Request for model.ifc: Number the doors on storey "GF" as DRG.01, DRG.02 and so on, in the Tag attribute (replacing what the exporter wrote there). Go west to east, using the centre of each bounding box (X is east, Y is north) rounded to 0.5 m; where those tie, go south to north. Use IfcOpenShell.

First a look at what the model holds.

```python
import ifcopenshell
import ifcopenshell.util.element
import ifcopenshell.util.placement

model = ifcopenshell.open("model.ifc")
print(model.schema)
storey = next(s for s in model.by_type("IfcBuildingStorey") if s.Name == "GF")
doors = [e for e in ifcopenshell.util.element.get_decomposition(storey) if e.is_a("IfcDoor")]
for e in sorted(doors, key=lambda e: e.id()):
    origin = ifcopenshell.util.placement.get_local_placement(e.ObjectPlacement)[:3, 3]
    print(e.id(), e.Tag, e.Name, origin.round(2) + 0.0, sep=" | ")
```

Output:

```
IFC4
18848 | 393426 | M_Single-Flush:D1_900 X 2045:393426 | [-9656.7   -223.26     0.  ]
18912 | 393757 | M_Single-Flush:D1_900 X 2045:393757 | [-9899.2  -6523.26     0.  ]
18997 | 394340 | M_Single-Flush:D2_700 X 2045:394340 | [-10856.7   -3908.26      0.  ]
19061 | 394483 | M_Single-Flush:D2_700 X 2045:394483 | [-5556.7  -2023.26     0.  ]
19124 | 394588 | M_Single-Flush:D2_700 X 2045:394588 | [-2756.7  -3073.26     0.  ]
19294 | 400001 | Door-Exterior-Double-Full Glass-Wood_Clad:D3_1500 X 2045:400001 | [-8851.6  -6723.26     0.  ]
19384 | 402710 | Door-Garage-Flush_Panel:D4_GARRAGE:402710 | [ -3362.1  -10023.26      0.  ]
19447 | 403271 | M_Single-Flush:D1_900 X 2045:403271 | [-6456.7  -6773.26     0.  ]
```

```python
import ifcopenshell
import ifcopenshell.geom
import ifcopenshell.util.element
import ifcopenshell.util.shape

model = ifcopenshell.open("model.ifc")
settings = ifcopenshell.geom.settings()
settings.set("use-world-coords", True)


def centre(element):
    shape = ifcopenshell.geom.create_shape(settings, element)
    return ifcopenshell.util.shape.get_bbox_centroid(shape.geometry)


storey = next(s for s in model.by_type("IfcBuildingStorey") if s.Name == "GF")
doors = [e for e in ifcopenshell.util.element.get_decomposition(storey) if e.is_a("IfcDoor")]

# Insertion points can sit at a corner or the storey origin, so sort by the geometry (in metres).
centres = {e: centre(e) for e in doors}
doors.sort(key=lambda e: (round(centres[e][0] / 0.5), centres[e][1]))

for i, e in enumerate(doors, start=1):
    number = f"DRG.{i:02d}"
    e.Tag = number
    print(e.id(), number)

model.write("model_rev.ifc")
```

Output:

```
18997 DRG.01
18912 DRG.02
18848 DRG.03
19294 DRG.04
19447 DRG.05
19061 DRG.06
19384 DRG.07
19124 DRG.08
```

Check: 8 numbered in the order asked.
